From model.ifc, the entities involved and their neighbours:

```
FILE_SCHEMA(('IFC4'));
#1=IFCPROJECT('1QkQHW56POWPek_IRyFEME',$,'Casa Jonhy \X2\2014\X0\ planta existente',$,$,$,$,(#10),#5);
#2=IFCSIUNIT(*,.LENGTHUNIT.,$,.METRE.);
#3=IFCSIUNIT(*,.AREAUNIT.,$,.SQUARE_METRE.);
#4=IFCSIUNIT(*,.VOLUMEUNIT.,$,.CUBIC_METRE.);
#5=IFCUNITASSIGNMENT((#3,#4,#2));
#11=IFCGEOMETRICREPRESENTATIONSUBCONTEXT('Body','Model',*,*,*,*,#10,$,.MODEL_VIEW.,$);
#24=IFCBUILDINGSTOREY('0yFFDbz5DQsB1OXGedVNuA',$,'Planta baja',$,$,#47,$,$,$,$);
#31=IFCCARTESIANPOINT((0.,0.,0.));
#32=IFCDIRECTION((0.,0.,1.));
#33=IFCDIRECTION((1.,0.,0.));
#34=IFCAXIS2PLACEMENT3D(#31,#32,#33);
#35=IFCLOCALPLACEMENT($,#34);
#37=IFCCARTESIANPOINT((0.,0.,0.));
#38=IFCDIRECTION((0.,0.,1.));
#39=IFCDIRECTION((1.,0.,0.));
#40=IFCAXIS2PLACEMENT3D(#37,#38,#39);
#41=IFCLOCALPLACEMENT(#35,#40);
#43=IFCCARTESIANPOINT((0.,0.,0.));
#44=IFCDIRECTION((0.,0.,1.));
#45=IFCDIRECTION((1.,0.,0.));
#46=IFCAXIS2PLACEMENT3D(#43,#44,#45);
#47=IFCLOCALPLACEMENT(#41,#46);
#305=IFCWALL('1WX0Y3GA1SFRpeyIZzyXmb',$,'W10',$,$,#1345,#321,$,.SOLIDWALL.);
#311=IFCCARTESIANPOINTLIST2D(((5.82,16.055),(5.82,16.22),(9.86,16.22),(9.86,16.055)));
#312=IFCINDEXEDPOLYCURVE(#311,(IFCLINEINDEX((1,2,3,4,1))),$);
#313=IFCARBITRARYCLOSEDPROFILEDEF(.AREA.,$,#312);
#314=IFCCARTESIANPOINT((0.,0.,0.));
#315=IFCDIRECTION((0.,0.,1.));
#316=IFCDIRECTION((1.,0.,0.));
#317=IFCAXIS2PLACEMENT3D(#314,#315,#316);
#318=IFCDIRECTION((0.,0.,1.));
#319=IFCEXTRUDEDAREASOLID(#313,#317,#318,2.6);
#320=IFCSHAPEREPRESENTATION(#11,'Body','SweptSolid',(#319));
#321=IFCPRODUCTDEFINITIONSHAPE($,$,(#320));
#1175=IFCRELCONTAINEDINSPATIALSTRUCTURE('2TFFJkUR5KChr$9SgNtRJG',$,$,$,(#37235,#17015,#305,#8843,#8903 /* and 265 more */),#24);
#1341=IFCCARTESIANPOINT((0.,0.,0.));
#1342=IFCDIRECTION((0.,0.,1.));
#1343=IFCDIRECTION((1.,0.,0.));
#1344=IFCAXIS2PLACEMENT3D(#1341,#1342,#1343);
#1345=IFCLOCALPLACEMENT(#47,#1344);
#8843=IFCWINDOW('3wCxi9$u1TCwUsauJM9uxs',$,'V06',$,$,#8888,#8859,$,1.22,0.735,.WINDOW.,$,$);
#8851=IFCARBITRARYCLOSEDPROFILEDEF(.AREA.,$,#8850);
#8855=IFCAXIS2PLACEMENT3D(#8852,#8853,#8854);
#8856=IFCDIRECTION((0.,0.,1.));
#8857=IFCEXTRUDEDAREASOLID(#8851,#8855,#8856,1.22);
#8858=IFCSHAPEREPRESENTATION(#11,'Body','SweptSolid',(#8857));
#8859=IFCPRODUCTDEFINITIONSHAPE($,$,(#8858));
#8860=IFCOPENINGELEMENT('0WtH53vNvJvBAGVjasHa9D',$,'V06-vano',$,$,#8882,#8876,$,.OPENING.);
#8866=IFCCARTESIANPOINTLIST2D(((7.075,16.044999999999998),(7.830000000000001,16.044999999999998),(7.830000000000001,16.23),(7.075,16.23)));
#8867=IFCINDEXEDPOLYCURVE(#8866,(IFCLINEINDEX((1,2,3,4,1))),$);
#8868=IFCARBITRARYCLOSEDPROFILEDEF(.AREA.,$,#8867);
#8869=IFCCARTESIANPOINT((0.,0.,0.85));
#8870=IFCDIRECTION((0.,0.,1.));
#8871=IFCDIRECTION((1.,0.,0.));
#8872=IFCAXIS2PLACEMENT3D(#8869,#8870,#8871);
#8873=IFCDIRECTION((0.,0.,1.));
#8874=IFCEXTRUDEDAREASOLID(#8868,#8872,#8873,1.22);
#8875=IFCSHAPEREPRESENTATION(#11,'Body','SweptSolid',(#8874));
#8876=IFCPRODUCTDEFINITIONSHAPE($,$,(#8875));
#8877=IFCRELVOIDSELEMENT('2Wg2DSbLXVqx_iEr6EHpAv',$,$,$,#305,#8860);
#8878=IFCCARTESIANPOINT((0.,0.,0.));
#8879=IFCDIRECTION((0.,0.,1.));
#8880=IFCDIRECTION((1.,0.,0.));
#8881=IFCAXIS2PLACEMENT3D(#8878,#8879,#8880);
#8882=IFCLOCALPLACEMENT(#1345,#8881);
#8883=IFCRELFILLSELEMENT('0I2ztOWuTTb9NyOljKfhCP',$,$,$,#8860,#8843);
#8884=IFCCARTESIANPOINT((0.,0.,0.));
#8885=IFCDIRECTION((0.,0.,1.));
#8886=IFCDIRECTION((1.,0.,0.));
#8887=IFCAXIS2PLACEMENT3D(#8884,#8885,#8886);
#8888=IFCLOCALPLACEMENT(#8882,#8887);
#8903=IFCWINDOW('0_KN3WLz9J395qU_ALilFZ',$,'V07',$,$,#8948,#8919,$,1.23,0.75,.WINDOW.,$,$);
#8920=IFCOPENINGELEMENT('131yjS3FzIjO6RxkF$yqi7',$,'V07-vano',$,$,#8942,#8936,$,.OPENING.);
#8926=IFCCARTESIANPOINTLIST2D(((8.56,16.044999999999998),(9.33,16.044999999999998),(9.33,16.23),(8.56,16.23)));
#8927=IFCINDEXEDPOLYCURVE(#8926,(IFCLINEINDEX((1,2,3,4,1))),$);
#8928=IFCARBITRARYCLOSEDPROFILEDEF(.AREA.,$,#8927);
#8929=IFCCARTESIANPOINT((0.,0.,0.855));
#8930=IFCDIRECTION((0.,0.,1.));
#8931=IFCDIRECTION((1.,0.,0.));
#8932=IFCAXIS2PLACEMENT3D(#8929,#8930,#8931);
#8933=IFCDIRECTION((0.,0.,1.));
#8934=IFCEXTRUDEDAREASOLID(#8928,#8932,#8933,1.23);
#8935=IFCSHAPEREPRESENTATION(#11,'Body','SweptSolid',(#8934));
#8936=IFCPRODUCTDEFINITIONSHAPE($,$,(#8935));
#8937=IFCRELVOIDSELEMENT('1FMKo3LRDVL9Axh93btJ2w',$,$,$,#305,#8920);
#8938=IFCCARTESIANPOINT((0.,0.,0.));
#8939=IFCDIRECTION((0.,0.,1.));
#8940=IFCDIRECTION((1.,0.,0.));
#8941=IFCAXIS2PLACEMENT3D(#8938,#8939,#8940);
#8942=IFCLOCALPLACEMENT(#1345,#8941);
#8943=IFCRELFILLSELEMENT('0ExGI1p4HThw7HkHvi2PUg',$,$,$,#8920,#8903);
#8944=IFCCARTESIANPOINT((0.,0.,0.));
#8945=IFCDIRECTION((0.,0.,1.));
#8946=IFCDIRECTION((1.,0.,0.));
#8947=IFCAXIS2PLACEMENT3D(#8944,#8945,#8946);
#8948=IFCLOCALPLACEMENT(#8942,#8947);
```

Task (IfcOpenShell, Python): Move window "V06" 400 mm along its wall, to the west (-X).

```python
import ifcopenshell
import ifcopenshell.api.geometry
import ifcopenshell.util.placement
import ifcopenshell.util.unit

model = ifcopenshell.open("model.ifc")
unit_scale = ifcopenshell.util.unit.calculate_unit_scale(model)

window = model.by_guid("3wCxi9$u1TCwUsauJM9uxs")
opening = window.FillsVoids[0].RelatingOpeningElement
wall = opening.VoidsElements[0].RelatingBuildingElement

wall_matrix = ifcopenshell.util.placement.get_local_placement(wall.ObjectPlacement)
shift = wall_matrix[:3, 0] * -0.4 / unit_scale
before = ifcopenshell.util.placement.get_local_placement(window.ObjectPlacement)[:3, 3].copy()

# The window is placed relative to its opening, so it follows when the opening moves.
matrix = ifcopenshell.util.placement.get_local_placement(opening.ObjectPlacement)
matrix[:3, 3] += shift
ifcopenshell.api.geometry.edit_object_placement(
    model, product=opening, matrix=matrix, is_si=False, should_transform_children=True
)

after = ifcopenshell.util.placement.get_local_placement(window.ObjectPlacement)[:3, 3]
print("window moved by", (after - before).round(3) + 0.0)

model.write("model-out.ifc")
```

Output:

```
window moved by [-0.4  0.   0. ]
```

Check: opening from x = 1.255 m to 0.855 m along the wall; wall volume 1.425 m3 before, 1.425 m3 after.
